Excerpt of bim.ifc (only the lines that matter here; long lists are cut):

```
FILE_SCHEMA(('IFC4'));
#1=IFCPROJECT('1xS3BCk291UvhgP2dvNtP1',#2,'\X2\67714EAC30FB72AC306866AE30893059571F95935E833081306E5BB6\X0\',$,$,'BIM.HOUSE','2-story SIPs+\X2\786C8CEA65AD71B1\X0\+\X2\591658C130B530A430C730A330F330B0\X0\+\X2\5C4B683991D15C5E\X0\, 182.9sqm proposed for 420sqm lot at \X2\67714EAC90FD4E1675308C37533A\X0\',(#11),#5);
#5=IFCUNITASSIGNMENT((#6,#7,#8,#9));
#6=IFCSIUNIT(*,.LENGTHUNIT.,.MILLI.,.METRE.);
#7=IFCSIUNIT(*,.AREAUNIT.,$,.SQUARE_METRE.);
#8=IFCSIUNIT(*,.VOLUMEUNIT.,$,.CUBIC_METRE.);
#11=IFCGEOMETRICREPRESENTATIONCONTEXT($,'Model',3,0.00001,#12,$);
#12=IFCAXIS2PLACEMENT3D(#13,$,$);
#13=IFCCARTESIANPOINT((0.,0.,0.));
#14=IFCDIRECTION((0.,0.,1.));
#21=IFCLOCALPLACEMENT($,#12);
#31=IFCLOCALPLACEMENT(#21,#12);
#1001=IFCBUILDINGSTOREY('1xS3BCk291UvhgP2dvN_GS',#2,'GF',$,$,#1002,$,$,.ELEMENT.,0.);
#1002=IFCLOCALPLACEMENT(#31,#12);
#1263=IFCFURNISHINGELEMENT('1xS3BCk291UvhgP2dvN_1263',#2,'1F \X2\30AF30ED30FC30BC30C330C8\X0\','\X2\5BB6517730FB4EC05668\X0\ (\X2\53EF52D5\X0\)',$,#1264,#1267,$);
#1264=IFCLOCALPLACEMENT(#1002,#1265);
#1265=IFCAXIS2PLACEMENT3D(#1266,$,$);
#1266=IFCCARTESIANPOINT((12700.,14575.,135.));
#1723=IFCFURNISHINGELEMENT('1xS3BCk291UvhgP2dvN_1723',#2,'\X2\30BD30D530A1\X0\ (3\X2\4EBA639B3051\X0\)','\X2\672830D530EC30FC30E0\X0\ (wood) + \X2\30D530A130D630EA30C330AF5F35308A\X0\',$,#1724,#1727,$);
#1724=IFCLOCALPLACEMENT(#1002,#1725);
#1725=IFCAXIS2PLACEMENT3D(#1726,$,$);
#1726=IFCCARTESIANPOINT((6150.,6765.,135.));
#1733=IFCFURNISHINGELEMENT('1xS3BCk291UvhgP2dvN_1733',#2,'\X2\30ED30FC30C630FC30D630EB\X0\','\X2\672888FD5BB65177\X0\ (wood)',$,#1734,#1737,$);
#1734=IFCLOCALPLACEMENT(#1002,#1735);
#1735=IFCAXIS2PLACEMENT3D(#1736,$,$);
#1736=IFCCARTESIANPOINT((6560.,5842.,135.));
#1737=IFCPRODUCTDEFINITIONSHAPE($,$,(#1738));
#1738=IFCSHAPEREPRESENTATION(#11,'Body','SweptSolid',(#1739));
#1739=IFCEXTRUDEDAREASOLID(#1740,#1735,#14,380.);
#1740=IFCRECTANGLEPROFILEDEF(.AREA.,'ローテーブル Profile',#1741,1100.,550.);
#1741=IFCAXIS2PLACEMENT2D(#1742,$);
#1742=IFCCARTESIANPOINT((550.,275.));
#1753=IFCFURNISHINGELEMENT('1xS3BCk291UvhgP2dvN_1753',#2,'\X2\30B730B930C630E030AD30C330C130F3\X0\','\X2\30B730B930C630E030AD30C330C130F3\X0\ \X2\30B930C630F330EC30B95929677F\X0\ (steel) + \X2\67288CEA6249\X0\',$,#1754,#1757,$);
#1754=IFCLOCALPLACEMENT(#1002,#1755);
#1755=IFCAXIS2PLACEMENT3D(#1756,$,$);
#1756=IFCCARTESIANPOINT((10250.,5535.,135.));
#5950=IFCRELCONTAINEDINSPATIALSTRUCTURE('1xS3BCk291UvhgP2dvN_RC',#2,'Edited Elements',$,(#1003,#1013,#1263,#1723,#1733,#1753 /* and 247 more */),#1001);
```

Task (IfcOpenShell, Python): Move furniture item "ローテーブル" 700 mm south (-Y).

```python
import ifcopenshell
import ifcopenshell.api.geometry
import ifcopenshell.util.placement
import ifcopenshell.util.unit

model = ifcopenshell.open("bim.ifc")
unit_scale = ifcopenshell.util.unit.calculate_unit_scale(model)

item = model.by_guid("1xS3BCk291UvhgP2dvN_1733")
matrix = ifcopenshell.util.placement.get_local_placement(item.ObjectPlacement)
matrix[1, 3] -= 0.7 / unit_scale
ifcopenshell.api.geometry.edit_object_placement(model, product=item, matrix=matrix, is_si=False)

print(ifcopenshell.util.placement.get_local_placement(item.ObjectPlacement).round(3) + 0.0)

model.write("bim_edited.ifc")
```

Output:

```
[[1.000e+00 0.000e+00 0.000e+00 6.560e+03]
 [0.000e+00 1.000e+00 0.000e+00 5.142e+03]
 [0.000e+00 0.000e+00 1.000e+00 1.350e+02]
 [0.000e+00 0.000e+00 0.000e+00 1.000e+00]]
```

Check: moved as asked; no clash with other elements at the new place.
